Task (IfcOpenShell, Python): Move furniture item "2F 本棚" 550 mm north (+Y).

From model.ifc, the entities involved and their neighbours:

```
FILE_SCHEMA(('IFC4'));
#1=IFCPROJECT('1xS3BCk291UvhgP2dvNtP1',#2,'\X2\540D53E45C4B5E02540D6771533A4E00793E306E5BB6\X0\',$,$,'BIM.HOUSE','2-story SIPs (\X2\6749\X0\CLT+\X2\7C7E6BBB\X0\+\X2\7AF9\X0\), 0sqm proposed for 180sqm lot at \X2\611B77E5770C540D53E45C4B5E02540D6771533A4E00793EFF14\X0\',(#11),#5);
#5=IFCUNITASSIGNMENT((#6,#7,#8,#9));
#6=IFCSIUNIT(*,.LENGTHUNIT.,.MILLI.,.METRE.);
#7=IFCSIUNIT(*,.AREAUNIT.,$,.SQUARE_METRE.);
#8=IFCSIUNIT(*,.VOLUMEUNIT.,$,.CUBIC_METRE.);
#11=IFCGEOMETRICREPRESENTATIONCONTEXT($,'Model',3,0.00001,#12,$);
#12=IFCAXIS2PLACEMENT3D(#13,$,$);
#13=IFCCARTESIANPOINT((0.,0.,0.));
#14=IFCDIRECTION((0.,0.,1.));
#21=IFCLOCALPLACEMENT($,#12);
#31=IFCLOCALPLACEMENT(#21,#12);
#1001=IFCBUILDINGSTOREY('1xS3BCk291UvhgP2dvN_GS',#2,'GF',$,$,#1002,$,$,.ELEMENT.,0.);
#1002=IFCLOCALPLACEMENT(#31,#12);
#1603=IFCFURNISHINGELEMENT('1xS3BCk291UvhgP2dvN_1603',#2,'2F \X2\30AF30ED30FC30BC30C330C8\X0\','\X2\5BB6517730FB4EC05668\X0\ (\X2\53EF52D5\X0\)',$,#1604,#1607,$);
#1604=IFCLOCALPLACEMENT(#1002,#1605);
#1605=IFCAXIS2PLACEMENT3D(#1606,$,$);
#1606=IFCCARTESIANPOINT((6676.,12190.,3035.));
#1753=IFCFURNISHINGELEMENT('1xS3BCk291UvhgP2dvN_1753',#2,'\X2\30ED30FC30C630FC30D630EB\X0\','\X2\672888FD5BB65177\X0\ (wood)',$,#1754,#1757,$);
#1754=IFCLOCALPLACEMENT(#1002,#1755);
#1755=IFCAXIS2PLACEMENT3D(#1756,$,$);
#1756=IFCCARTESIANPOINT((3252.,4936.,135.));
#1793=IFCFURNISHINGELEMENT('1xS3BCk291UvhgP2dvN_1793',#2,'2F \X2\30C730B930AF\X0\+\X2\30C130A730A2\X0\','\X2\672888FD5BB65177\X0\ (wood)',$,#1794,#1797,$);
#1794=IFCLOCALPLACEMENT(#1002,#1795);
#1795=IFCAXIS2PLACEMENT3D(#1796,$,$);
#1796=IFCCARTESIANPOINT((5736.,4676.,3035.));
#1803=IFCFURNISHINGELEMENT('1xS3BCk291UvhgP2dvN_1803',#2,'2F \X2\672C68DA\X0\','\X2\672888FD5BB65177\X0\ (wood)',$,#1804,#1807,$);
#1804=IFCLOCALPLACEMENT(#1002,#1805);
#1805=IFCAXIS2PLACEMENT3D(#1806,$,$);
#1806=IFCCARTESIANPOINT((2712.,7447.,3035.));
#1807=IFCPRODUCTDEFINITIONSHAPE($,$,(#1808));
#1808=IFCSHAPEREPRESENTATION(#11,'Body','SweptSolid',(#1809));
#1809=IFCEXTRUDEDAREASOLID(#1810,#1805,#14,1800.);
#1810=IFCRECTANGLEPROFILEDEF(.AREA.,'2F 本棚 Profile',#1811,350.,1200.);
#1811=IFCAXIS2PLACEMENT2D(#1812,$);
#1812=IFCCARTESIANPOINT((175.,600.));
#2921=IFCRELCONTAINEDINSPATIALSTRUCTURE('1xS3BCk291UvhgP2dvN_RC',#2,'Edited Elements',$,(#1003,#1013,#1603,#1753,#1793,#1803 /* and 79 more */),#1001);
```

```python
import ifcopenshell
import ifcopenshell.api.geometry
import ifcopenshell.util.placement

model = ifcopenshell.open("model.ifc")

item = model.by_id(1803)
matrix = ifcopenshell.util.placement.get_local_placement(item.ObjectPlacement)
matrix[1, 3] += 550.0
ifcopenshell.api.geometry.edit_object_placement(model, product=item, matrix=matrix, is_si=False)

print(ifcopenshell.util.placement.get_local_placement(item.ObjectPlacement).round(3) + 0.0)

model.write("model_v2.ifc")
```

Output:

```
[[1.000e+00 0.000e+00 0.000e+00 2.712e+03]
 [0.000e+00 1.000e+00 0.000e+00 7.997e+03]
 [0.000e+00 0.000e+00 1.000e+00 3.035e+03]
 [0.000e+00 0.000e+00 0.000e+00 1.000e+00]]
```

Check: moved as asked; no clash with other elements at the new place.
